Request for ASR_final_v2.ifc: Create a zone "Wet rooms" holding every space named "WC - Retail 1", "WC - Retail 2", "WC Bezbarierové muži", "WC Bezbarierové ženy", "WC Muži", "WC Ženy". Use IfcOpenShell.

First a look at what the model holds.

```python
import ifcopenshell

model = ifcopenshell.open("ASR_final_v2.ifc")
print(model.schema)
seen = {}
for space in model.by_type("IfcSpace"):
    seen[space.LongName] = seen.get(space.LongName, 0) + 1
for name, count in sorted(seen.items(), key=str):
    print(count, "x", name)
print("zones:", [z.Name for z in model.by_type("IfcZone")][:20])
```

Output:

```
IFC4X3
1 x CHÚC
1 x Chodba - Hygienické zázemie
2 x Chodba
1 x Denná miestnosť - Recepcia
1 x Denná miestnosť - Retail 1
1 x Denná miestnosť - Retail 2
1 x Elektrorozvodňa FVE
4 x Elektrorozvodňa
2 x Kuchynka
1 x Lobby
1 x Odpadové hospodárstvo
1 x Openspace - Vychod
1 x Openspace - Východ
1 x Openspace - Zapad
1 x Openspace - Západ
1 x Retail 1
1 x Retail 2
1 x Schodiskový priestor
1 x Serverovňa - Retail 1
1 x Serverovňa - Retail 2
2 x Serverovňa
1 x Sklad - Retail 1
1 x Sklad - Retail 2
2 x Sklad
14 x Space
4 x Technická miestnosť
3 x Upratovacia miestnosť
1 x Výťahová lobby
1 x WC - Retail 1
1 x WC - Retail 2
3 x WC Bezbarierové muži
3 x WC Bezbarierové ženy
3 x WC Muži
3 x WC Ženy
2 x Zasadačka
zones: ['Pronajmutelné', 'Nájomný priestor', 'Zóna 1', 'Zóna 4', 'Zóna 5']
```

```python
import ifcopenshell
import ifcopenshell.api.group
import ifcopenshell.api.root

model = ifcopenshell.open("ASR_final_v2.ifc")

names = {"WC - Retail 1", "WC - Retail 2", "WC Bezbarierové muži", "WC Bezbarierové ženy", "WC Muži", "WC Ženy"}
spaces = [s for s in model.by_type("IfcSpace") if s.LongName in names]

zone = ifcopenshell.api.root.create_entity(model, ifc_class="IfcZone", name="Wet rooms")
ifcopenshell.api.group.assign_group(model, products=spaces, group=zone)
print(len(spaces), "spaces in", zone.Name)

model.write("ASR_final_v2_rev.ifc")
```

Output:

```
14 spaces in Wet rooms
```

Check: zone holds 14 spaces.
